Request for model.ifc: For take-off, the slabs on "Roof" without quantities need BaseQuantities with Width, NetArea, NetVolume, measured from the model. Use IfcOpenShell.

First a look at what the model holds.

```python
import ifcopenshell
import ifcopenshell.util.element
import ifcopenshell.util.unit

model = ifcopenshell.open("model.ifc")
print(model.schema)
for unit_type in ("LENGTHUNIT", "AREAUNIT", "VOLUMEUNIT"):
    print(unit_type, ifcopenshell.util.unit.calculate_unit_scale(model, unit_type))
storey = next(s for s in model.by_type("IfcBuildingStorey") if s.Name == "Roof")
slabs = [e for e in ifcopenshell.util.element.get_decomposition(storey) if e.is_a("IfcSlab")]
for e in sorted(slabs, key=lambda e: e.id()):
    print(e.id(), e.is_a(), e.Name, list(ifcopenshell.util.element.get_psets(e, qtos_only=True)), sep=" | ")
```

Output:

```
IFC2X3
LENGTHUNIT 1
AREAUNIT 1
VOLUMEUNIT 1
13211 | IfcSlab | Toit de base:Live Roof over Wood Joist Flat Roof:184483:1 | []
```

```python
import ifcopenshell
import ifcopenshell.api.pset
import ifcopenshell.geom
import ifcopenshell.util.element
import ifcopenshell.util.shape
import ifcopenshell.util.unit

model = ifcopenshell.open("model.ifc")
unit_scale = ifcopenshell.util.unit.calculate_unit_scale(model)
area_scale = ifcopenshell.util.unit.calculate_unit_scale(model, "AREAUNIT")
volume_scale = ifcopenshell.util.unit.calculate_unit_scale(model, "VOLUMEUNIT")
settings = ifcopenshell.geom.settings()

storey = next(s for s in model.by_type("IfcBuildingStorey") if s.Name == "Roof")
slabs = [e for e in ifcopenshell.util.element.get_decomposition(storey) if e.is_a("IfcSlab")]

for e in sorted(slabs, key=lambda e: e.id()):
    if ifcopenshell.util.element.get_psets(e, qtos_only=True, should_inherit=False):
        continue
    # Geometry comes back in metres, in the element's own axes.
    shape = ifcopenshell.geom.create_shape(settings, e)
    values = {
        "Width": ifcopenshell.util.shape.get_z(shape.geometry) / unit_scale,
        "NetArea": ifcopenshell.util.shape.get_footprint_area(shape.geometry) / area_scale,
        "NetVolume": ifcopenshell.util.shape.get_volume(shape.geometry) / volume_scale,
    }
    qto = ifcopenshell.api.pset.add_qto(model, product=e, name="BaseQuantities")
    ifcopenshell.api.pset.edit_qto(model, qto=qto, properties=values)
    print(e.id(), {k: round(v, 3) for k, v in values.items()})

model.write("model_edited.ifc")
```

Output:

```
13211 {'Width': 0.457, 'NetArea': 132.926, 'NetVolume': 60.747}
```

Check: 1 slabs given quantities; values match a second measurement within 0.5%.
